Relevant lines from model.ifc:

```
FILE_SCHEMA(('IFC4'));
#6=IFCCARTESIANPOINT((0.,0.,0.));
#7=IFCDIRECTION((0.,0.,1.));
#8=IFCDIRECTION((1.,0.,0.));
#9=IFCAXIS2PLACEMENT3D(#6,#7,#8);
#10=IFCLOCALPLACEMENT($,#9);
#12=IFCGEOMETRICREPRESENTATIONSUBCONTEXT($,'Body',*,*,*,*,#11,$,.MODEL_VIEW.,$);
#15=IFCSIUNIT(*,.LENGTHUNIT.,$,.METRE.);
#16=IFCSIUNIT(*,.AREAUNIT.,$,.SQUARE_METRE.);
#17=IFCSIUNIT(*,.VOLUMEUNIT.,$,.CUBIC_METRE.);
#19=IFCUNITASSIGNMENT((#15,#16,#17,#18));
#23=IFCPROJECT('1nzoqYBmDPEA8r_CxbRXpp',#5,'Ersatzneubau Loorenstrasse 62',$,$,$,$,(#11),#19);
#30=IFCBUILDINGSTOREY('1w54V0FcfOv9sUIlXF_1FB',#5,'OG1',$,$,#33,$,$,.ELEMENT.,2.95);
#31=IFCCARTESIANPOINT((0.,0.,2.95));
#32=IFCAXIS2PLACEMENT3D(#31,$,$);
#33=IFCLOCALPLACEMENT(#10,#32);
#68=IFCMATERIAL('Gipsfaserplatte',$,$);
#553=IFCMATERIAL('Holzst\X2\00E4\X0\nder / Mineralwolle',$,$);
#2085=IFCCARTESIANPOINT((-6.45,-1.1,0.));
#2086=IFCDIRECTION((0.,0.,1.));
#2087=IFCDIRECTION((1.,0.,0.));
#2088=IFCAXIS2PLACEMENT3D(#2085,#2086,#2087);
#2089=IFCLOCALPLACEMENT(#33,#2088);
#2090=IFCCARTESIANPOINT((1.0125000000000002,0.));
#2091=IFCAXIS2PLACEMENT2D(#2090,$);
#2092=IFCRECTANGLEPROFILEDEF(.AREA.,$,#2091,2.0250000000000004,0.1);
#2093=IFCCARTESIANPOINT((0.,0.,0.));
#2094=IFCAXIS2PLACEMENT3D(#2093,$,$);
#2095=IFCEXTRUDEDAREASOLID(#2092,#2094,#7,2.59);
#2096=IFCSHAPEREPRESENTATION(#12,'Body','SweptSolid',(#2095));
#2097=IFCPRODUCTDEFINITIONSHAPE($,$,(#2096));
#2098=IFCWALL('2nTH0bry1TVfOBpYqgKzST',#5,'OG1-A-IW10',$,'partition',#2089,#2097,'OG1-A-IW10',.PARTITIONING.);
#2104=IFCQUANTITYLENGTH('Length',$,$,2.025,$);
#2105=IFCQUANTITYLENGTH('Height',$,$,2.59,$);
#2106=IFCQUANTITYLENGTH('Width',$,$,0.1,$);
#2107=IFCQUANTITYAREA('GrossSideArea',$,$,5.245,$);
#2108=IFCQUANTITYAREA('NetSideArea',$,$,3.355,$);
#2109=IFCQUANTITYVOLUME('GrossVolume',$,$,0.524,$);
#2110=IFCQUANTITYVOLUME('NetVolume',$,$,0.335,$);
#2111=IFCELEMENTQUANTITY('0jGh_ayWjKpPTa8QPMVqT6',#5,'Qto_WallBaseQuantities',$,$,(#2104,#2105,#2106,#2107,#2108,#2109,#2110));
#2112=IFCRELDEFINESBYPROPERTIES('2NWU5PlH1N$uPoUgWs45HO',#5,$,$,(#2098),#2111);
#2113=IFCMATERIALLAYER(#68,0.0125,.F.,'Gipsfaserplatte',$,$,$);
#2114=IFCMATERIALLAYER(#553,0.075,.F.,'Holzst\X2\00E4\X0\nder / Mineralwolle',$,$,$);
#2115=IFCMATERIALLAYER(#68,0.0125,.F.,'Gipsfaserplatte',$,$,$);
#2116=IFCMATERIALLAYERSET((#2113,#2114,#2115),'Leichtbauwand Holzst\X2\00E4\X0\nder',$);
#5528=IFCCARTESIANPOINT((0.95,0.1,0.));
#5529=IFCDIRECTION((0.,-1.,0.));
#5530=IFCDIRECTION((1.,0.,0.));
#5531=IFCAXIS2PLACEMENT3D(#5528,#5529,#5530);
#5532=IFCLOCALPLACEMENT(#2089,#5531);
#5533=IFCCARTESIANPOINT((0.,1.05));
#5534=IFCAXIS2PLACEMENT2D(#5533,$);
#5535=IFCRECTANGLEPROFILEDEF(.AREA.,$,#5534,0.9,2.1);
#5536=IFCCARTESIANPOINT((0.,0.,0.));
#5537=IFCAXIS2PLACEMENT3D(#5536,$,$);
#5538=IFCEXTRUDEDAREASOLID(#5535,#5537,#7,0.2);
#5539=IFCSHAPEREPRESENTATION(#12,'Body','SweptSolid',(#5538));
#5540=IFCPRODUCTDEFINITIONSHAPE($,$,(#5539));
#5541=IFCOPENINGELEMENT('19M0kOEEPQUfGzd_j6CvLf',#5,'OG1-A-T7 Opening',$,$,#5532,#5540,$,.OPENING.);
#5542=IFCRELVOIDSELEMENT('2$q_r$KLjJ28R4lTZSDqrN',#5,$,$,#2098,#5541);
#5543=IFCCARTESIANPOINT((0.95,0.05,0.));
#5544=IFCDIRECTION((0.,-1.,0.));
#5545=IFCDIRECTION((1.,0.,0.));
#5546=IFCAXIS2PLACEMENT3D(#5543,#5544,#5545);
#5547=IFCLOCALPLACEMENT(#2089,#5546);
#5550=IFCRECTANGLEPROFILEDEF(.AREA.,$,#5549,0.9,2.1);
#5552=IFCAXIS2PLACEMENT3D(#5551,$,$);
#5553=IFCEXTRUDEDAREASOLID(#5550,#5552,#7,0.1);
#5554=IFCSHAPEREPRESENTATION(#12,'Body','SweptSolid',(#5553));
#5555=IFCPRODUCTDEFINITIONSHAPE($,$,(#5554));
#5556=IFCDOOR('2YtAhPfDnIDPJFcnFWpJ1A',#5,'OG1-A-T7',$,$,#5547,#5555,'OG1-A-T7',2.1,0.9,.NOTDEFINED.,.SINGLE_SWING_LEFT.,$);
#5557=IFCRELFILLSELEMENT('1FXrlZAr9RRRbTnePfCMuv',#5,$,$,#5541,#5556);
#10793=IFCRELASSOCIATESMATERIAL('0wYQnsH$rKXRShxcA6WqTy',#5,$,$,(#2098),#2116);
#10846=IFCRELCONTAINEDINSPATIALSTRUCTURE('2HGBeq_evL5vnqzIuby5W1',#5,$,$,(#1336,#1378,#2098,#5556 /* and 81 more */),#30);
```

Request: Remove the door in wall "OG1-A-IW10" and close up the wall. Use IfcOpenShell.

```python
import ifcopenshell
import ifcopenshell.api.feature
import ifcopenshell.api.pset
import ifcopenshell.api.root
import ifcopenshell.geom
import ifcopenshell.util.element
import ifcopenshell.util.shape
import ifcopenshell.util.unit

model = ifcopenshell.open("model.ifc")
area_scale = ifcopenshell.util.unit.calculate_unit_scale(model, "AREAUNIT")
volume_scale = ifcopenshell.util.unit.calculate_unit_scale(model, "VOLUMEUNIT")
settings = ifcopenshell.geom.settings()


def volume(element):
    """Net volume in cubic metres, openings subtracted."""
    shape = ifcopenshell.geom.create_shape(settings, element)
    return ifcopenshell.util.shape.get_volume(shape.geometry)


door = model.by_id(5556)
opening = door.FillsVoids[0].RelatingOpeningElement
wall = opening.VoidsElements[0].RelatingBuildingElement
before = volume(wall)

ifcopenshell.api.root.remove_product(model, product=door)
ifcopenshell.api.feature.remove_feature(model, feature=opening)

after = volume(wall)
thickness = 0.1  # wall thickness in metres

# Update the wall's stored quantities.
qto = model.by_id(ifcopenshell.util.element.get_pset(wall, "Qto_WallBaseQuantities", should_inherit=False)["id"])
ifcopenshell.api.pset.edit_qto(model, qto=qto, properties={
    "NetSideArea": after / thickness / area_scale,
    "NetVolume": after / volume_scale,
})

print(f"wall volume {before:.3f} -> {after:.3f} m3")

model.write("model_updated.ifc")
```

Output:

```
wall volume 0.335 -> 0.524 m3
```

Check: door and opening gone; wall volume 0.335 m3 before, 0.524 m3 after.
